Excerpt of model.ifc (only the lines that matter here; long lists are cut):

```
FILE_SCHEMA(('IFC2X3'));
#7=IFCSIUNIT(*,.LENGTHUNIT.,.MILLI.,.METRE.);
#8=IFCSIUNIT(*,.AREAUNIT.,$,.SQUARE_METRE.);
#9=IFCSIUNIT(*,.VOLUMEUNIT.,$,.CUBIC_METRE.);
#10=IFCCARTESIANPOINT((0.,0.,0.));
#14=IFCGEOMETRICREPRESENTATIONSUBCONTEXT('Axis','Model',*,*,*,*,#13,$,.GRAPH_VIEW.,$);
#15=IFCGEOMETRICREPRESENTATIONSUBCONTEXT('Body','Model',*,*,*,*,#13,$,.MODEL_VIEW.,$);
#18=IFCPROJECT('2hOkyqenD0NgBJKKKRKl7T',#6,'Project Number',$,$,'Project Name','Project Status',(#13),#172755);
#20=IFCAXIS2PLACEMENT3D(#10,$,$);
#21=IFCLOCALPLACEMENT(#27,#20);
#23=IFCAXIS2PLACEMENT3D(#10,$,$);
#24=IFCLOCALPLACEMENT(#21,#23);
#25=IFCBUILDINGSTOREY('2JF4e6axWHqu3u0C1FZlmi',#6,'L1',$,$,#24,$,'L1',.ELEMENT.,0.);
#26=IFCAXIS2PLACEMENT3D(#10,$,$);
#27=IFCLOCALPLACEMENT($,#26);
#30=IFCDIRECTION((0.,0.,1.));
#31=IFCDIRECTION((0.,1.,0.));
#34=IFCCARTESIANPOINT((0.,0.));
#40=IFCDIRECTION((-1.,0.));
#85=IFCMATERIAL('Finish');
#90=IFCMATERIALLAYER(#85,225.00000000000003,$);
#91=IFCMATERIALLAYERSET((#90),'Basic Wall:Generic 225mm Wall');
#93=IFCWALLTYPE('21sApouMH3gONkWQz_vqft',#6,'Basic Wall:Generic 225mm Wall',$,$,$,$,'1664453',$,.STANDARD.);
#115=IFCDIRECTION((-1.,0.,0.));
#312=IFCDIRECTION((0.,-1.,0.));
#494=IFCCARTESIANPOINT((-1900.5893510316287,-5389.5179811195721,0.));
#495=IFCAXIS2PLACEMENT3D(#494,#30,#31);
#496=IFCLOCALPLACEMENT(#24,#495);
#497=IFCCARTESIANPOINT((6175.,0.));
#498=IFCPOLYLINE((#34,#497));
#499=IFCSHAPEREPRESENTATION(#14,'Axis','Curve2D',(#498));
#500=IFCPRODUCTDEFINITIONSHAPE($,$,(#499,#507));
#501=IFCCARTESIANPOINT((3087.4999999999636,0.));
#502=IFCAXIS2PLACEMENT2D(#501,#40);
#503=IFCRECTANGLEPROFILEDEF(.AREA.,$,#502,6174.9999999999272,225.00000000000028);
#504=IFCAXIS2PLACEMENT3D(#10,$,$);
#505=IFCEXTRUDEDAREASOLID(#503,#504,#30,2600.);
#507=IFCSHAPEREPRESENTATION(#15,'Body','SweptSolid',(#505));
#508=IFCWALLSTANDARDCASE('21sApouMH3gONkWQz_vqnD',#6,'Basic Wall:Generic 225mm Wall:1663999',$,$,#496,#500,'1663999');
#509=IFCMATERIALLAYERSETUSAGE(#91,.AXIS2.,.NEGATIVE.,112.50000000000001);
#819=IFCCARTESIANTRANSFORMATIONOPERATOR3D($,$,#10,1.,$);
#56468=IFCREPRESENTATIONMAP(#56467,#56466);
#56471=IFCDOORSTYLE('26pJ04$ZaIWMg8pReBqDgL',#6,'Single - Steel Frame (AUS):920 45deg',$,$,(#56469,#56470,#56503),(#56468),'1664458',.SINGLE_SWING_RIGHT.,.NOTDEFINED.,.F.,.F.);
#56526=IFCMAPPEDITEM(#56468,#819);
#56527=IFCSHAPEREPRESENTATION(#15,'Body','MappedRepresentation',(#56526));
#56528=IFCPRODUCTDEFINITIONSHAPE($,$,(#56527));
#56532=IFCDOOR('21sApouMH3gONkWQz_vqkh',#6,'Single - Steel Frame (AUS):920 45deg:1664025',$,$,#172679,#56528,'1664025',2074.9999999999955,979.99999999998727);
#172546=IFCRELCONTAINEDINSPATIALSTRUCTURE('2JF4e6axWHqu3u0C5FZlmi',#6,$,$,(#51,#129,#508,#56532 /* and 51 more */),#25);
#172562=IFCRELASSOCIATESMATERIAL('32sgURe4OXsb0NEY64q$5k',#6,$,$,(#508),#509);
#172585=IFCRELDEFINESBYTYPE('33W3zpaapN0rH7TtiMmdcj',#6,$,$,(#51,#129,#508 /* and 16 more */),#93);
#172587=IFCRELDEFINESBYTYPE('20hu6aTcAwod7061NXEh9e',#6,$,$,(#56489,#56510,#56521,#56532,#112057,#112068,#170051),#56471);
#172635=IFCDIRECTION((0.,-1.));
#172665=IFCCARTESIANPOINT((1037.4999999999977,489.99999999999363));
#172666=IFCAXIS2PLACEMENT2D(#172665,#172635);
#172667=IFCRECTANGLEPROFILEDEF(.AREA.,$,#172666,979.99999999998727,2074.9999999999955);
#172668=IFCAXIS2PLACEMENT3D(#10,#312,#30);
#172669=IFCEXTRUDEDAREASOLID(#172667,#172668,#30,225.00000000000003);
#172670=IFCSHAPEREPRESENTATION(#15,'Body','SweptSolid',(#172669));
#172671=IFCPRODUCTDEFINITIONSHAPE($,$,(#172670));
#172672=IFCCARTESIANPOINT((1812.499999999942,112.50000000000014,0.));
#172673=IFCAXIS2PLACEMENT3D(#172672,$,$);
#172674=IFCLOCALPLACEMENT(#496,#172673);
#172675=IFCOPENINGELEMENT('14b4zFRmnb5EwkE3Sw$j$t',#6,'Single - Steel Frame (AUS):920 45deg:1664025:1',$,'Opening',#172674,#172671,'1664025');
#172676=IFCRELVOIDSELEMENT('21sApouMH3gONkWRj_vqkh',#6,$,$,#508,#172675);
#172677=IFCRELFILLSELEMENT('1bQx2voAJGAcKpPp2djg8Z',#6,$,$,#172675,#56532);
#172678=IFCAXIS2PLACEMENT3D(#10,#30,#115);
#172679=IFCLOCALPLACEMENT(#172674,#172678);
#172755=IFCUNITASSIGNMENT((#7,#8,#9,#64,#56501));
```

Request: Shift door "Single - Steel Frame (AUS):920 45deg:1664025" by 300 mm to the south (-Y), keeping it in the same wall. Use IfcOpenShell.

```python
import ifcopenshell
import ifcopenshell.api.geometry
import ifcopenshell.util.placement

model = ifcopenshell.open("model.ifc")

door = model.by_guid("21sApouMH3gONkWQz_vqkh")
opening = door.FillsVoids[0].RelatingOpeningElement
wall = opening.VoidsElements[0].RelatingBuildingElement

wall_matrix = ifcopenshell.util.placement.get_local_placement(wall.ObjectPlacement)
shift = wall_matrix[:3, 0] * -300.0
before = ifcopenshell.util.placement.get_local_placement(door.ObjectPlacement)[:3, 3].copy()

# The door is placed relative to its opening, so it follows when the opening moves.
matrix = ifcopenshell.util.placement.get_local_placement(opening.ObjectPlacement)
matrix[:3, 3] += shift
ifcopenshell.api.geometry.edit_object_placement(
    model, product=opening, matrix=matrix, is_si=False, should_transform_children=True
)

after = ifcopenshell.util.placement.get_local_placement(door.ObjectPlacement)[:3, 3]
print("door moved by", (after - before).round(3) + 0.0)

model.write("model-out.ifc")
```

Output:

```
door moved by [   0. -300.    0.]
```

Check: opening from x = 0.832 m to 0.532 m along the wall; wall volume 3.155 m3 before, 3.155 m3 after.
